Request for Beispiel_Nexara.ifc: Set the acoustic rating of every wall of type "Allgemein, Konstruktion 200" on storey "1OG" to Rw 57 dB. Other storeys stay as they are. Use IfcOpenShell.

First a look at what the model holds.

```python
import ifcopenshell
import ifcopenshell.util.element

model = ifcopenshell.open("Beispiel_Nexara.ifc")
print(model.schema)
storey = next(s for s in model.by_type("IfcBuildingStorey") if s.Name == "1OG")
walls = [e for e in ifcopenshell.util.element.get_decomposition(storey) if e.is_a("IfcWall")]
seen = {}
for e in walls:
    element_type = ifcopenshell.util.element.get_type(e)
    key = (element_type.Name if element_type != e and element_type else None, ifcopenshell.util.element.get_pset(e, "Pset_WallCommon", "AcousticRating"))
    seen[key] = seen.get(key, 0) + 1
for (name, value), count in sorted(seen.items(), key=str):
    print(count, "x", name, "|", value)
```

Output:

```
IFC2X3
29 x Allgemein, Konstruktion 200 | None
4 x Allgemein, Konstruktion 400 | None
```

```python
import ifcopenshell
import ifcopenshell.api.pset
import ifcopenshell.util.element

model = ifcopenshell.open("Beispiel_Nexara.ifc")

storey = next(s for s in model.by_type("IfcBuildingStorey") if s.Name == "1OG")
walls = [e for e in ifcopenshell.util.element.get_decomposition(storey) if e.is_a("IfcWall")]

count = 0
for e in walls:
    element_type = ifcopenshell.util.element.get_type(e)
    if element_type in (None, e) or element_type.Name != "Allgemein, Konstruktion 200":
        continue
    # add_pset returns the element's existing set when there is one.
    pset = ifcopenshell.api.pset.add_pset(model, product=e, name="Pset_WallCommon")
    ifcopenshell.api.pset.edit_pset(model, pset=pset, properties={"AcousticRating": "Rw 57 dB"})
    count += 1

print(count, "walls updated")

model.write("Beispiel_Nexara-out.ifc")
```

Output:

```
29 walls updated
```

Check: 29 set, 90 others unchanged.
